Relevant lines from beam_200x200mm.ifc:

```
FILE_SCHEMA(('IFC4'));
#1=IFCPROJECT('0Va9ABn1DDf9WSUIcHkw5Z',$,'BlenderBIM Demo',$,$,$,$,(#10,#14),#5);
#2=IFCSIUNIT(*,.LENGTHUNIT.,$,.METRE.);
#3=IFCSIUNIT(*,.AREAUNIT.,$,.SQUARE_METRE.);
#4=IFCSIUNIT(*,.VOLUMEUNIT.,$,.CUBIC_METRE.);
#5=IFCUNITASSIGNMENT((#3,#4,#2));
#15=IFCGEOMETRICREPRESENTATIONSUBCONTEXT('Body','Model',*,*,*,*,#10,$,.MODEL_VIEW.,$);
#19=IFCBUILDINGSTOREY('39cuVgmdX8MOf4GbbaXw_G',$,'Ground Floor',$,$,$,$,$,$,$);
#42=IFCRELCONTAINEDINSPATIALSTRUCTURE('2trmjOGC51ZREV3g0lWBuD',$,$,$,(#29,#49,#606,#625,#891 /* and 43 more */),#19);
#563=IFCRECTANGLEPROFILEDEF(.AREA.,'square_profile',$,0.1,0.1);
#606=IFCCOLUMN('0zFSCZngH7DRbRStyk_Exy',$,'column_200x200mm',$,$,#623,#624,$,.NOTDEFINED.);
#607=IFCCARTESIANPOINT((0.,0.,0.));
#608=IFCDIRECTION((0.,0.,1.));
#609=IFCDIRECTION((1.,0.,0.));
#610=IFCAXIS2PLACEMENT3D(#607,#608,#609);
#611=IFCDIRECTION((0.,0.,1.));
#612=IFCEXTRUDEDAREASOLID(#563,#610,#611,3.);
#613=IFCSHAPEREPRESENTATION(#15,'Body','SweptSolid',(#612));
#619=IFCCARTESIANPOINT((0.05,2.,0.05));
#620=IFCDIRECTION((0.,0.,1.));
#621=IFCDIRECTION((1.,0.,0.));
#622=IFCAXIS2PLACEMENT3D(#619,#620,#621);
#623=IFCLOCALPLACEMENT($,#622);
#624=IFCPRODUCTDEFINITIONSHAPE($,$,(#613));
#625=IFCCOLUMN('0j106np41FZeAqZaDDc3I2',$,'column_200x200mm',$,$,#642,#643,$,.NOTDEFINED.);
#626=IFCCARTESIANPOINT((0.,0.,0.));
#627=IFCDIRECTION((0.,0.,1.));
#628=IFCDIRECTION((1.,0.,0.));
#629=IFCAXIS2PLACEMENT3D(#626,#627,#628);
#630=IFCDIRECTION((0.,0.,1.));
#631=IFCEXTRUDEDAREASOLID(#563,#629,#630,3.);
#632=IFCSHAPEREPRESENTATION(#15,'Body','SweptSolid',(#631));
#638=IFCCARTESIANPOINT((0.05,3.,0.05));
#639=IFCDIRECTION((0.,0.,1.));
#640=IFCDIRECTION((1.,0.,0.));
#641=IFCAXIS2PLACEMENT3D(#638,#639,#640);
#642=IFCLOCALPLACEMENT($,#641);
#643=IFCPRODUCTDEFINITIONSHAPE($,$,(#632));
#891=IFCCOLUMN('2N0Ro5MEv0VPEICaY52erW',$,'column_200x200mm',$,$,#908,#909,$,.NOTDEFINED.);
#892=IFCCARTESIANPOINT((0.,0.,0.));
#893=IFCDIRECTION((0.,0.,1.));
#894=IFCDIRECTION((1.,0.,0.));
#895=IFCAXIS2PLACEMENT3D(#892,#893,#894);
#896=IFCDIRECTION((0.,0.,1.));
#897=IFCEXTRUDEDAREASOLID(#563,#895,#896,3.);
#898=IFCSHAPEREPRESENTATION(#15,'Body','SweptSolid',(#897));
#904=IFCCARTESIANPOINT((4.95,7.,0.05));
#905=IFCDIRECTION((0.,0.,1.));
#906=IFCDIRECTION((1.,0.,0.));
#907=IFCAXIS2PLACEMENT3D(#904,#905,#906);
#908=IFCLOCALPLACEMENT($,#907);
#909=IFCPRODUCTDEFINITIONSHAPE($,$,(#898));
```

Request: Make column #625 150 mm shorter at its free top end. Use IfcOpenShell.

```python
import ifcopenshell
import ifcopenshell.util.representation
import ifcopenshell.util.unit

model = ifcopenshell.open("beam_200x200mm.ifc")
unit_scale = ifcopenshell.util.unit.calculate_unit_scale(model)

member = model.by_id(625)
change = -0.15 / unit_scale

# The extrusion runs towards the end named, so only its depth changes.
body = ifcopenshell.util.representation.get_representation(member, "Model", "Body")
solid = body.Items[0]
old_length = solid.Depth
solid.Depth += change

print(f"length {old_length:g} -> {solid.Depth:g}")

model.write("beam_200x200mm_rev.ifc")
```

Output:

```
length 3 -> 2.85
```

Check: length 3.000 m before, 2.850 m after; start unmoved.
